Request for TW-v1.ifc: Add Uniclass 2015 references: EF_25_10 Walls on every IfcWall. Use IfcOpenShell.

First a look at what the model holds.

```python
import ifcopenshell

model = ifcopenshell.open("TW-v1.ifc")
print(model.schema)
print("classifications:", [c.Name for c in model.by_type("IfcClassification")])
for ifc_class in ("IfcDoor", "IfcRoof", "IfcStair", "IfcWall", "IfcWindow"):
    print(ifc_class, len(model.by_type(ifc_class)))
```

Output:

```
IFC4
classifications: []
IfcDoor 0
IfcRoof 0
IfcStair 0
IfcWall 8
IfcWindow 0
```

```python
import ifcopenshell
import ifcopenshell.api.classification

model = ifcopenshell.open("TW-v1.ifc")

system = ifcopenshell.api.classification.add_classification(model, classification="Uniclass 2015")

codes = {
    "IfcWall": ("EF_25_10", "Walls"),
}
for ifc_class, (code, name) in codes.items():
    products = model.by_type(ifc_class)
    ifcopenshell.api.classification.add_reference(
        model, products=products, classification=system, identification=code, name=name
    )
    print(code, len(products))

model.write("TW-v1_updated.ifc")
```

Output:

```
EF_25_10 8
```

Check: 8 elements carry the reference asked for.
